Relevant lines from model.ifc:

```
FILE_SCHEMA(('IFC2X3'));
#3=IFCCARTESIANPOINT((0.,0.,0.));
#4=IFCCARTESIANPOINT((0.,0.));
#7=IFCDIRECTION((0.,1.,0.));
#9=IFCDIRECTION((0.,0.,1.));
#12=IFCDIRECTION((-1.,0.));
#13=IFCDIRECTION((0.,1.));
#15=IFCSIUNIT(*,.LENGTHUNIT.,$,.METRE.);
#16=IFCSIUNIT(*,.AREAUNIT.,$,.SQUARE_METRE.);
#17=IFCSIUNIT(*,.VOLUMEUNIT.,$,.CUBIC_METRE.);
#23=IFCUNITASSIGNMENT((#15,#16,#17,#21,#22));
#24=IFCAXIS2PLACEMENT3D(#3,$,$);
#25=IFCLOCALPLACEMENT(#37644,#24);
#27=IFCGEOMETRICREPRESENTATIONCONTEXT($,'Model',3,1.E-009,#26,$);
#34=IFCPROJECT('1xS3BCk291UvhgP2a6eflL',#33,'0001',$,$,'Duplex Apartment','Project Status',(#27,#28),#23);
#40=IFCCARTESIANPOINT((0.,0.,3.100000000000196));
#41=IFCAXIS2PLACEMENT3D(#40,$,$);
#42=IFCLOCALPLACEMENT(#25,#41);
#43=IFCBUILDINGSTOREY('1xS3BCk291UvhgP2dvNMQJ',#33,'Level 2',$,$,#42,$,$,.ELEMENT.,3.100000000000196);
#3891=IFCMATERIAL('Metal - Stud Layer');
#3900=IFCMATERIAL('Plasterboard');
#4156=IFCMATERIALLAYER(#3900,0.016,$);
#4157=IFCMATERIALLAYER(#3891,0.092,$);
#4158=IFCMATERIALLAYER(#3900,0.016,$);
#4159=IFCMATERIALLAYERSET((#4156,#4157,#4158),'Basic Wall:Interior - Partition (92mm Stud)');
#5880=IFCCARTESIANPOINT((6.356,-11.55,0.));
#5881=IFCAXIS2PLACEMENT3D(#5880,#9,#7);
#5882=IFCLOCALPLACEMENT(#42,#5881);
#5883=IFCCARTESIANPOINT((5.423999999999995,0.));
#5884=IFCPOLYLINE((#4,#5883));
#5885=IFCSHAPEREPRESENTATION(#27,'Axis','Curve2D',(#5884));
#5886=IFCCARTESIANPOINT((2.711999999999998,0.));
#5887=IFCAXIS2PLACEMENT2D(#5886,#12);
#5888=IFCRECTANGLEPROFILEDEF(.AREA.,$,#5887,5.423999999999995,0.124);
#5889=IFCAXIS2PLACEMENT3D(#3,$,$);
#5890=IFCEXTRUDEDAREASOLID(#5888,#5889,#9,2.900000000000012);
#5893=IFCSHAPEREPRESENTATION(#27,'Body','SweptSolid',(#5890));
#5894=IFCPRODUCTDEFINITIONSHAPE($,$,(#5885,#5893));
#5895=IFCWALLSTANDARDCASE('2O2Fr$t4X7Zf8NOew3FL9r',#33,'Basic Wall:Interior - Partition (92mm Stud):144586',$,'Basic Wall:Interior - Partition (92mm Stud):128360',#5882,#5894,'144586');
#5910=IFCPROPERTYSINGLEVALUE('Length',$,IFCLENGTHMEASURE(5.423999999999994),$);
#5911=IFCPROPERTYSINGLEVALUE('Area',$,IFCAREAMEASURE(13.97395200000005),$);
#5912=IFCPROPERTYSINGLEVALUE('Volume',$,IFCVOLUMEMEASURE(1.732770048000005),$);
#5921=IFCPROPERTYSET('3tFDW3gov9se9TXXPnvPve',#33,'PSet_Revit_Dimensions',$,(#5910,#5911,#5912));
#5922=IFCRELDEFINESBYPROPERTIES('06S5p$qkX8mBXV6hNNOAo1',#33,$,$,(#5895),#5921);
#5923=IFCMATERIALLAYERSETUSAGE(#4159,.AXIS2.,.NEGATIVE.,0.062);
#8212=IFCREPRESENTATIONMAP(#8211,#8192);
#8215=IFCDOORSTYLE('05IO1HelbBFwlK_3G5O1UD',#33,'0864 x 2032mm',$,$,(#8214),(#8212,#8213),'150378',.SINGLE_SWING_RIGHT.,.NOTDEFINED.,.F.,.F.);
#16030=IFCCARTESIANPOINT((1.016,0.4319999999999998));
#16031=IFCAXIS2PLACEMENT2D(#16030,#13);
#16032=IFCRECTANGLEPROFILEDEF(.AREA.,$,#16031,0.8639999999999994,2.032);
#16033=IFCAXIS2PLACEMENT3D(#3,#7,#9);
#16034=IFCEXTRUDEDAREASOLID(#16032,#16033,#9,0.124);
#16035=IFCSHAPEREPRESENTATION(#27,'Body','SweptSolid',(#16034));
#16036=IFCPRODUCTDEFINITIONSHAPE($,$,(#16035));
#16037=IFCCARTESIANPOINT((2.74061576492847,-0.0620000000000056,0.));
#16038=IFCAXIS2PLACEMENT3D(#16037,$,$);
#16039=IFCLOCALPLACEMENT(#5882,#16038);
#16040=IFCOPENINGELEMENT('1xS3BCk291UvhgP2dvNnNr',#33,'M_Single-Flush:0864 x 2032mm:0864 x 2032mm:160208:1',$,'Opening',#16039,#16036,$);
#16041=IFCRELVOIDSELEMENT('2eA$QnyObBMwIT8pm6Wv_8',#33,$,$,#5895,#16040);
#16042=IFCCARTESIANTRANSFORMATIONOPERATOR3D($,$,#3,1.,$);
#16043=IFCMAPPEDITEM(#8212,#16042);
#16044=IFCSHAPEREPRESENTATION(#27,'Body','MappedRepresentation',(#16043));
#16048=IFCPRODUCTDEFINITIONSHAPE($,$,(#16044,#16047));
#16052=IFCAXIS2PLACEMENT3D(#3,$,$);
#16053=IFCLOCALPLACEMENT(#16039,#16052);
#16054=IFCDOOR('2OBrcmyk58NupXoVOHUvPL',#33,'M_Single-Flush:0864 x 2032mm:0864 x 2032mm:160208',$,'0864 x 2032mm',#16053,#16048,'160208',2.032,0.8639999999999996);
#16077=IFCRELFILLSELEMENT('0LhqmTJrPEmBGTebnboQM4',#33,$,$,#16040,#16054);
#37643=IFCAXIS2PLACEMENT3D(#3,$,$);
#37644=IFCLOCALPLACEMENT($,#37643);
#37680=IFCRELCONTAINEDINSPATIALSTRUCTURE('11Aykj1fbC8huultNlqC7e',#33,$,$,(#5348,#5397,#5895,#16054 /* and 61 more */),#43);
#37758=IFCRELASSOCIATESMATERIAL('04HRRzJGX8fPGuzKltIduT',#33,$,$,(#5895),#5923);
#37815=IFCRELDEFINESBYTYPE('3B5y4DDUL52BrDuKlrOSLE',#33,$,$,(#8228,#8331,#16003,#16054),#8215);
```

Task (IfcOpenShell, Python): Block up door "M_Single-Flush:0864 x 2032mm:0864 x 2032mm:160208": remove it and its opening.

```python
import ifcopenshell
import ifcopenshell.api.feature
import ifcopenshell.api.pset
import ifcopenshell.api.root
import ifcopenshell.geom
import ifcopenshell.util.element
import ifcopenshell.util.shape
import ifcopenshell.util.unit

model = ifcopenshell.open("model.ifc")
area_scale = ifcopenshell.util.unit.calculate_unit_scale(model, "AREAUNIT")
volume_scale = ifcopenshell.util.unit.calculate_unit_scale(model, "VOLUMEUNIT")
settings = ifcopenshell.geom.settings()


def volume(element):
    """Net volume in cubic metres, openings subtracted."""
    shape = ifcopenshell.geom.create_shape(settings, element)
    return ifcopenshell.util.shape.get_volume(shape.geometry)


door = model.by_id(16054)
opening = door.FillsVoids[0].RelatingOpeningElement
wall = opening.VoidsElements[0].RelatingBuildingElement
before = volume(wall)

ifcopenshell.api.root.remove_product(model, product=door)
ifcopenshell.api.feature.remove_feature(model, feature=opening)

after = volume(wall)
thickness = 0.124  # wall thickness in metres

# Update the wall's stored quantities.
pset = model.by_id(ifcopenshell.util.element.get_pset(wall, "PSet_Revit_Dimensions", should_inherit=False)["id"])
ifcopenshell.api.pset.edit_pset(model, pset=pset, properties={
    "Area": model.create_entity("IfcAreaMeasure", after / thickness / area_scale),
    "Volume": model.create_entity("IfcVolumeMeasure", after / volume_scale),
})

print(f"wall volume {before:.3f} -> {after:.3f} m3")

model.write("model_updated.ifc")
```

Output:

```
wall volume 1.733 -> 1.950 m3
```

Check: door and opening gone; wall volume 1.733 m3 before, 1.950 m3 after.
